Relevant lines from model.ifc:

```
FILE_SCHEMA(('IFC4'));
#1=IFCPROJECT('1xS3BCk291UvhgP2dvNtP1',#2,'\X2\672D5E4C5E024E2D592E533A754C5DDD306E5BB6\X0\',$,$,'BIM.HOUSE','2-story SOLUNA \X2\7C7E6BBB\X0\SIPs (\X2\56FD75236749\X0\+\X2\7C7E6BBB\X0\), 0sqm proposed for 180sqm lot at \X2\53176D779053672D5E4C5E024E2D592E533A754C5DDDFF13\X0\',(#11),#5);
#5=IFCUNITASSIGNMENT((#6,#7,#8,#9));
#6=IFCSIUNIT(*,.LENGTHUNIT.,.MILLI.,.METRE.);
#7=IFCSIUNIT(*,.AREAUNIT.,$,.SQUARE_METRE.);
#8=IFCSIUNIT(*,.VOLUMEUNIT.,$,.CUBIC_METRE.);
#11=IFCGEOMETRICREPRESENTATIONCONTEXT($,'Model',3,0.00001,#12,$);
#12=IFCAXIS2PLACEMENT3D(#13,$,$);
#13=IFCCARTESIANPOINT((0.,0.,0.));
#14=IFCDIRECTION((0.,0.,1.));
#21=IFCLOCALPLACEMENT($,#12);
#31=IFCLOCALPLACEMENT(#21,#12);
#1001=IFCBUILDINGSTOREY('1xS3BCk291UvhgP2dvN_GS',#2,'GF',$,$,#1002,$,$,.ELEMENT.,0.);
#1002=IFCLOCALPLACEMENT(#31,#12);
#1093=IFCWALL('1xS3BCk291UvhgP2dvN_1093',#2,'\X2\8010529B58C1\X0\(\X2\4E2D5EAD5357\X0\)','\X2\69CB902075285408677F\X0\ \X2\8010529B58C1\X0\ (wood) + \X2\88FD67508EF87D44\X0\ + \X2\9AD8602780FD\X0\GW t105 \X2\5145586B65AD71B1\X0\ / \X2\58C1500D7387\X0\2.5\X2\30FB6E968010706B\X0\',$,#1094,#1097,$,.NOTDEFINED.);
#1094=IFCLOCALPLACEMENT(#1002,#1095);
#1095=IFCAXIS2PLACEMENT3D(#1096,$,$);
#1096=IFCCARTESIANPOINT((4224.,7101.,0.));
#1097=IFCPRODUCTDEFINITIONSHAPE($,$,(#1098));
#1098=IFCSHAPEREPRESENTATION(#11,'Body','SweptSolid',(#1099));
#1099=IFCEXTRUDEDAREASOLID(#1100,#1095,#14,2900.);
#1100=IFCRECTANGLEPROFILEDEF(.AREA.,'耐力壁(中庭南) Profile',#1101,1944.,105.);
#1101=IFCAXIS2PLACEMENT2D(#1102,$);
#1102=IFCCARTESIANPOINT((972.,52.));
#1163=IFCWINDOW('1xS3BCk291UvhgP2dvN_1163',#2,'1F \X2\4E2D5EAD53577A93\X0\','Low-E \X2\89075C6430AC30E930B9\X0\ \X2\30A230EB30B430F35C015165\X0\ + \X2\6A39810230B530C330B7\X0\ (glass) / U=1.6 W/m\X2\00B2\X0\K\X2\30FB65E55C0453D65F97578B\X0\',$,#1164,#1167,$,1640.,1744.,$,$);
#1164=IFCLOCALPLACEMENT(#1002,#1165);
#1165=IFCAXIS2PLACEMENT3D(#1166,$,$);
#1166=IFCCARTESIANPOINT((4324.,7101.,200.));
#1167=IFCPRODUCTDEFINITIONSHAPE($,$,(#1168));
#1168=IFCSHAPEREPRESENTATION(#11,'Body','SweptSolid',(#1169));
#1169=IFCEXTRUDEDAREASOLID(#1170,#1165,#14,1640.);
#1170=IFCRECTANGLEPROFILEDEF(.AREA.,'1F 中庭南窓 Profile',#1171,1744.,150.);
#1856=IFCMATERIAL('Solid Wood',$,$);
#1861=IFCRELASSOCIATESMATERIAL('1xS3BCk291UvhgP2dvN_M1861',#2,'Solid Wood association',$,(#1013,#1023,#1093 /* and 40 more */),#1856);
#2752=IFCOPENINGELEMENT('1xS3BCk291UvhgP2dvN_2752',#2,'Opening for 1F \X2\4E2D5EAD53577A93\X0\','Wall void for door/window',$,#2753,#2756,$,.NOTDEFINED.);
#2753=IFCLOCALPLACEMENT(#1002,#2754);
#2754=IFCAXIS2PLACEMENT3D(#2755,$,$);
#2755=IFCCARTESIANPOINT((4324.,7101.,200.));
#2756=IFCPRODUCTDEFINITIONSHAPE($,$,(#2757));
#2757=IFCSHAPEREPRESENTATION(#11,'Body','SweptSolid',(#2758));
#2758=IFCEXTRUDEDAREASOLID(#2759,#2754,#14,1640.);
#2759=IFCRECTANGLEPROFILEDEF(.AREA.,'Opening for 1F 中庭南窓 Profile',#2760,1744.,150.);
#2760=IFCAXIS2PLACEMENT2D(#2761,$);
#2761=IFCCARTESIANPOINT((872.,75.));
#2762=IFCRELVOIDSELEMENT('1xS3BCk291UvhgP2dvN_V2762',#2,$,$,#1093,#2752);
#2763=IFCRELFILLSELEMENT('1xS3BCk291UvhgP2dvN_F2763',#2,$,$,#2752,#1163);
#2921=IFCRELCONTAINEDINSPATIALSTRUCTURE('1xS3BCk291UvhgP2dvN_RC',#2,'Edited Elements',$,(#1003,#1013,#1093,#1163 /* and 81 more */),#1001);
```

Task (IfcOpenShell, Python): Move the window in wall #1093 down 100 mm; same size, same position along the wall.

```python
import numpy as np
import ifcopenshell
import ifcopenshell.api.geometry
import ifcopenshell.util.placement
import ifcopenshell.util.unit

model = ifcopenshell.open("model.ifc")
unit_scale = ifcopenshell.util.unit.calculate_unit_scale(model)

window = model.by_guid("1xS3BCk291UvhgP2dvN_1163")
opening = window.FillsVoids[0].RelatingOpeningElement
dz = -0.1 / unit_scale

shift = np.array([0.0, 0.0, dz])
# The window is not placed relative to its opening, so move both.
for product in (opening, window):
    matrix = ifcopenshell.util.placement.get_local_placement(product.ObjectPlacement)
    matrix[:3, 3] += shift
    ifcopenshell.api.geometry.edit_object_placement(model, product=product, matrix=matrix, is_si=False)

print(f"moved by {dz * unit_scale:+.3f} m")

model.write("model-out.ifc")
```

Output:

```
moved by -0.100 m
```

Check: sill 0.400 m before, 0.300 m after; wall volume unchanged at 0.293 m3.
